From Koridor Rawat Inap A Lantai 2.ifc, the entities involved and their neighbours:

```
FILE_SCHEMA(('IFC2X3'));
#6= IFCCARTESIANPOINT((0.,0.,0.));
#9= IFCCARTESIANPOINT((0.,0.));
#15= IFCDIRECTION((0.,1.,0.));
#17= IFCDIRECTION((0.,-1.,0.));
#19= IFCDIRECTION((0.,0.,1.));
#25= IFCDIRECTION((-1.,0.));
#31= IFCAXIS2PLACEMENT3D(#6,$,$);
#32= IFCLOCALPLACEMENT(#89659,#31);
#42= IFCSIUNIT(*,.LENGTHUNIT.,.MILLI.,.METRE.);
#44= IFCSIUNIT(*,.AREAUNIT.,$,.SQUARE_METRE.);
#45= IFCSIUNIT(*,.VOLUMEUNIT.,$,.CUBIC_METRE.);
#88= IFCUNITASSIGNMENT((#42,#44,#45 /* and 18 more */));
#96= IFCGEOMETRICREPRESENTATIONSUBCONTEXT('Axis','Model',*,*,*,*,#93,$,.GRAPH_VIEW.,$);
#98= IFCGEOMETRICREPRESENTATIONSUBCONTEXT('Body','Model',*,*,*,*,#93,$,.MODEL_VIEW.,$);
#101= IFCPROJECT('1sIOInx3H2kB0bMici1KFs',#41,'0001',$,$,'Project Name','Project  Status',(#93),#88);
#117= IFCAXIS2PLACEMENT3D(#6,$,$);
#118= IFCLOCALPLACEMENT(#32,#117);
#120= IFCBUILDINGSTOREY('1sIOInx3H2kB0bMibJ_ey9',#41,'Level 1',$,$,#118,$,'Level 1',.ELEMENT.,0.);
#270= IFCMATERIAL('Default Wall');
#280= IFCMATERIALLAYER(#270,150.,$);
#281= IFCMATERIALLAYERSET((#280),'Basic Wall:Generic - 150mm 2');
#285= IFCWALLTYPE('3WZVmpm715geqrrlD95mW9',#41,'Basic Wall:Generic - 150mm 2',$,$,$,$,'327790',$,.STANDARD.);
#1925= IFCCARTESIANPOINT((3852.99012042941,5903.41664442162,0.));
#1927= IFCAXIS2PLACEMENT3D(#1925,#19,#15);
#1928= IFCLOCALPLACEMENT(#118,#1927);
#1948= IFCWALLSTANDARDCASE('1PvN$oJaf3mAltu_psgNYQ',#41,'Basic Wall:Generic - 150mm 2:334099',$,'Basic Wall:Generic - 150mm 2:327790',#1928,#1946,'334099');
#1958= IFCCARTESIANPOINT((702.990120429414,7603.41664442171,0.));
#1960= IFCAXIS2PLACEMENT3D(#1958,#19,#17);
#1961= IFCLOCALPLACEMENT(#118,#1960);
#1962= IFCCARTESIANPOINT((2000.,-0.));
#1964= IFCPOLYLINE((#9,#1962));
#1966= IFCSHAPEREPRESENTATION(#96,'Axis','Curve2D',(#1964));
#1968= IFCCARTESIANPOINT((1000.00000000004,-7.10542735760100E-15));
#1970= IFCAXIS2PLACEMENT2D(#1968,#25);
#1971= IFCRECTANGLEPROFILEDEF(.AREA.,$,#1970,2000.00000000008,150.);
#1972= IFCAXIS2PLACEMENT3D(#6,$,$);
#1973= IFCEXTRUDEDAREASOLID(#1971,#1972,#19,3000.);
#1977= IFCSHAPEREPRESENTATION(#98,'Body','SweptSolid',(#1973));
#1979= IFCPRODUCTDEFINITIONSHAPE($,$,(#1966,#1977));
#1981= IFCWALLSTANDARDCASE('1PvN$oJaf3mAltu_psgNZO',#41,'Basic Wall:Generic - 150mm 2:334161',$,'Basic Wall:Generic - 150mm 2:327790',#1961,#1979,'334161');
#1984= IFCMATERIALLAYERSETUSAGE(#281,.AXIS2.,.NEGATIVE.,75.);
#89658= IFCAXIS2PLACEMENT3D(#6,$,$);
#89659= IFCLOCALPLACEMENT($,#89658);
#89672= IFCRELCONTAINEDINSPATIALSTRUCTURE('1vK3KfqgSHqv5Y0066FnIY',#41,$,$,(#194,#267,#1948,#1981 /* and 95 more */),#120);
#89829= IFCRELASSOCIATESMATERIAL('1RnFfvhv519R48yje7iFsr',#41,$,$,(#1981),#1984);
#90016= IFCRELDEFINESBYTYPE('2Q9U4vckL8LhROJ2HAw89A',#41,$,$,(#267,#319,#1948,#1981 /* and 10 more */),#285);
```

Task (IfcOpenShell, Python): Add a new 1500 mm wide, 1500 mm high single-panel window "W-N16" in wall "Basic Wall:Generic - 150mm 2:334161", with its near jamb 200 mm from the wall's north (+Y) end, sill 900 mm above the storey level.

```python
import numpy as np
import ifcopenshell
import ifcopenshell.api.feature
import ifcopenshell.api.geometry
import ifcopenshell.api.root
import ifcopenshell.api.spatial
import ifcopenshell.api.type
import ifcopenshell.geom
import ifcopenshell.util.element
import ifcopenshell.util.placement
import ifcopenshell.util.representation
import ifcopenshell.util.shape
import ifcopenshell.util.unit

model = ifcopenshell.open("Koridor Rawat Inap A Lantai 2.ifc")
unit_scale = ifcopenshell.util.unit.calculate_unit_scale(model)
settings = ifcopenshell.geom.settings()


def volume(element):
    """Net volume in cubic metres, openings subtracted."""
    shape = ifcopenshell.geom.create_shape(settings, element)
    return ifcopenshell.util.shape.get_volume(shape.geometry)


wall = model.by_id(1981)
storey = ifcopenshell.util.element.get_container(wall, ifc_class="IfcBuildingStorey")
context = ifcopenshell.util.representation.get_context(model, "Model", "Body", "MODEL_VIEW")
before = volume(wall)

width, height, from_end, sill = 1.5, 1.5, 0.2, 0.9  # metres

# The wall runs along its own X axis, and the end named is its -X end.
wall_shape = ifcopenshell.geom.create_shape(settings, wall)
x, y, z = ifcopenshell.util.shape.get_vertices(wall_shape.geometry).T
start = x.min() + from_end
face, thickness = float(y.min()), float(y.max() - y.min())
wall_matrix = ifcopenshell.util.placement.get_local_placement(wall.ObjectPlacement)
level = ifcopenshell.util.placement.get_local_placement(storey.ObjectPlacement)[2, 3]


def in_wall(x, y):
    """Placement at x, y metres in the wall's axes, at sill height."""
    matrix = wall_matrix.copy()
    matrix[:, 3] = wall_matrix @ np.array([x / unit_scale, y / unit_scale, 0.0, 1.0])
    matrix[2, 3] = level + sill / unit_scale
    return matrix


# Opening: a box that overshoots both wall faces by 50 mm.
opening = ifcopenshell.api.root.create_entity(model, ifc_class="IfcOpeningElement")
box = ifcopenshell.api.geometry.add_wall_representation(
    model, context=context, length=width, height=height, thickness=thickness + 0.1
)
ifcopenshell.api.geometry.assign_representation(model, product=opening, representation=box)
ifcopenshell.api.geometry.edit_object_placement(model, product=opening, matrix=in_wall(start, face - 0.05), is_si=False)
ifcopenshell.api.feature.add_feature(model, feature=opening, element=wall)

window = ifcopenshell.api.root.create_entity(model, ifc_class="IfcWindow", name="W-N16")
window.OverallWidth, window.OverallHeight = width / unit_scale, height / unit_scale
body = ifcopenshell.api.geometry.add_window_representation(
    model,
    context=context,
    overall_width=window.OverallWidth,
    overall_height=window.OverallHeight,
    partition_type="SINGLE_PANEL",
)
ifcopenshell.api.geometry.assign_representation(model, product=window, representation=body)
ifcopenshell.api.spatial.assign_container(model, products=[window], relating_structure=storey)
fills = ifcopenshell.api.feature.add_filling(model, opening=opening, element=window)
fills.OwnerHistory = window.OwnerHistory  # required in IFC2X3

# IFC2X3 keeps the operation on the window style.
style = ifcopenshell.api.root.create_entity(model, ifc_class="IfcWindowStyle", name="W-N16")
style.OperationType, style.ConstructionType = "SINGLE_PANEL", "NOTDEFINED"
style.ParameterTakesPrecedence = style.Sizeable = False
ifcopenshell.api.type.assign_type(model, related_objects=[window], relating_type=style)

# Centre the window in the wall's thickness.
ifcopenshell.api.geometry.edit_object_placement(model, product=window, matrix=in_wall(start, face), is_si=False)
window_shape = ifcopenshell.geom.create_shape(settings, window)
depth = ifcopenshell.util.shape.get_vertices(window_shape.geometry)[:, 1]
offset = face + thickness / 2 - (depth.min() + depth.max()) / 2
ifcopenshell.api.geometry.edit_object_placement(model, product=window, matrix=in_wall(start, offset), is_si=False)

after = volume(wall)

print(f"wall volume {before:.3f} -> {after:.3f} m3")

model.write("Koridor Rawat Inap A Lantai 2-out.ifc")
```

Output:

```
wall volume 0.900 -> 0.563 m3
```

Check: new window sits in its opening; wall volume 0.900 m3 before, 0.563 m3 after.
